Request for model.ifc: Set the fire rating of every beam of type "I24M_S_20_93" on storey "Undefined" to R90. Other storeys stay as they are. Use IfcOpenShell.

First a look at what the model holds.

```python
import ifcopenshell
import ifcopenshell.util.element

model = ifcopenshell.open("model.ifc")
print(model.schema)
storey = next(s for s in model.by_type("IfcBuildingStorey") if s.Name == "Undefined")
beams = [e for e in ifcopenshell.util.element.get_decomposition(storey) if e.is_a("IfcBeam")]
seen = {}
for e in beams:
    element_type = ifcopenshell.util.element.get_type(e)
    key = (element_type.Name if element_type != e and element_type else None, ifcopenshell.util.element.get_pset(e, "Pset_BeamCommon", "FireRating"))
    seen[key] = seen.get(key, 0) + 1
for (name, value), count in sorted(seen.items(), key=str):
    print(count, "x", name, "|", value)
```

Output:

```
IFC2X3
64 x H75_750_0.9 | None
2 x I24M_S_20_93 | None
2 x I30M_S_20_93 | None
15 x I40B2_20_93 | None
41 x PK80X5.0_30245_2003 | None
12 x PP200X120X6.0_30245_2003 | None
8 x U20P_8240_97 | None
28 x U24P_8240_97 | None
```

```python
import ifcopenshell
import ifcopenshell.api.pset
import ifcopenshell.util.element

model = ifcopenshell.open("model.ifc")

storey = next(s for s in model.by_type("IfcBuildingStorey") if s.Name == "Undefined")
beams = [e for e in ifcopenshell.util.element.get_decomposition(storey) if e.is_a("IfcBeam")]

count = 0
for e in beams:
    element_type = ifcopenshell.util.element.get_type(e)
    if element_type in (None, e) or element_type.Name != "I24M_S_20_93":
        continue
    found = ifcopenshell.util.element.get_pset(e, "Pset_BeamCommon", should_inherit=False)
    if found:
        pset = model.by_id(found["id"])
        if len(ifcopenshell.util.element.get_elements_by_pset(pset)) > 1:
            pset = ifcopenshell.api.pset.unshare_pset(model, products=[e], pset=pset)[0]
    else:
        pset = ifcopenshell.api.pset.add_pset(model, product=e, name="Pset_BeamCommon")
    ifcopenshell.api.pset.edit_pset(model, pset=pset, properties={"FireRating": "R90"})
    count += 1

print(count, "beams updated")

model.write("model_rev.ifc")
```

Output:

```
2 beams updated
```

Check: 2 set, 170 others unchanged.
